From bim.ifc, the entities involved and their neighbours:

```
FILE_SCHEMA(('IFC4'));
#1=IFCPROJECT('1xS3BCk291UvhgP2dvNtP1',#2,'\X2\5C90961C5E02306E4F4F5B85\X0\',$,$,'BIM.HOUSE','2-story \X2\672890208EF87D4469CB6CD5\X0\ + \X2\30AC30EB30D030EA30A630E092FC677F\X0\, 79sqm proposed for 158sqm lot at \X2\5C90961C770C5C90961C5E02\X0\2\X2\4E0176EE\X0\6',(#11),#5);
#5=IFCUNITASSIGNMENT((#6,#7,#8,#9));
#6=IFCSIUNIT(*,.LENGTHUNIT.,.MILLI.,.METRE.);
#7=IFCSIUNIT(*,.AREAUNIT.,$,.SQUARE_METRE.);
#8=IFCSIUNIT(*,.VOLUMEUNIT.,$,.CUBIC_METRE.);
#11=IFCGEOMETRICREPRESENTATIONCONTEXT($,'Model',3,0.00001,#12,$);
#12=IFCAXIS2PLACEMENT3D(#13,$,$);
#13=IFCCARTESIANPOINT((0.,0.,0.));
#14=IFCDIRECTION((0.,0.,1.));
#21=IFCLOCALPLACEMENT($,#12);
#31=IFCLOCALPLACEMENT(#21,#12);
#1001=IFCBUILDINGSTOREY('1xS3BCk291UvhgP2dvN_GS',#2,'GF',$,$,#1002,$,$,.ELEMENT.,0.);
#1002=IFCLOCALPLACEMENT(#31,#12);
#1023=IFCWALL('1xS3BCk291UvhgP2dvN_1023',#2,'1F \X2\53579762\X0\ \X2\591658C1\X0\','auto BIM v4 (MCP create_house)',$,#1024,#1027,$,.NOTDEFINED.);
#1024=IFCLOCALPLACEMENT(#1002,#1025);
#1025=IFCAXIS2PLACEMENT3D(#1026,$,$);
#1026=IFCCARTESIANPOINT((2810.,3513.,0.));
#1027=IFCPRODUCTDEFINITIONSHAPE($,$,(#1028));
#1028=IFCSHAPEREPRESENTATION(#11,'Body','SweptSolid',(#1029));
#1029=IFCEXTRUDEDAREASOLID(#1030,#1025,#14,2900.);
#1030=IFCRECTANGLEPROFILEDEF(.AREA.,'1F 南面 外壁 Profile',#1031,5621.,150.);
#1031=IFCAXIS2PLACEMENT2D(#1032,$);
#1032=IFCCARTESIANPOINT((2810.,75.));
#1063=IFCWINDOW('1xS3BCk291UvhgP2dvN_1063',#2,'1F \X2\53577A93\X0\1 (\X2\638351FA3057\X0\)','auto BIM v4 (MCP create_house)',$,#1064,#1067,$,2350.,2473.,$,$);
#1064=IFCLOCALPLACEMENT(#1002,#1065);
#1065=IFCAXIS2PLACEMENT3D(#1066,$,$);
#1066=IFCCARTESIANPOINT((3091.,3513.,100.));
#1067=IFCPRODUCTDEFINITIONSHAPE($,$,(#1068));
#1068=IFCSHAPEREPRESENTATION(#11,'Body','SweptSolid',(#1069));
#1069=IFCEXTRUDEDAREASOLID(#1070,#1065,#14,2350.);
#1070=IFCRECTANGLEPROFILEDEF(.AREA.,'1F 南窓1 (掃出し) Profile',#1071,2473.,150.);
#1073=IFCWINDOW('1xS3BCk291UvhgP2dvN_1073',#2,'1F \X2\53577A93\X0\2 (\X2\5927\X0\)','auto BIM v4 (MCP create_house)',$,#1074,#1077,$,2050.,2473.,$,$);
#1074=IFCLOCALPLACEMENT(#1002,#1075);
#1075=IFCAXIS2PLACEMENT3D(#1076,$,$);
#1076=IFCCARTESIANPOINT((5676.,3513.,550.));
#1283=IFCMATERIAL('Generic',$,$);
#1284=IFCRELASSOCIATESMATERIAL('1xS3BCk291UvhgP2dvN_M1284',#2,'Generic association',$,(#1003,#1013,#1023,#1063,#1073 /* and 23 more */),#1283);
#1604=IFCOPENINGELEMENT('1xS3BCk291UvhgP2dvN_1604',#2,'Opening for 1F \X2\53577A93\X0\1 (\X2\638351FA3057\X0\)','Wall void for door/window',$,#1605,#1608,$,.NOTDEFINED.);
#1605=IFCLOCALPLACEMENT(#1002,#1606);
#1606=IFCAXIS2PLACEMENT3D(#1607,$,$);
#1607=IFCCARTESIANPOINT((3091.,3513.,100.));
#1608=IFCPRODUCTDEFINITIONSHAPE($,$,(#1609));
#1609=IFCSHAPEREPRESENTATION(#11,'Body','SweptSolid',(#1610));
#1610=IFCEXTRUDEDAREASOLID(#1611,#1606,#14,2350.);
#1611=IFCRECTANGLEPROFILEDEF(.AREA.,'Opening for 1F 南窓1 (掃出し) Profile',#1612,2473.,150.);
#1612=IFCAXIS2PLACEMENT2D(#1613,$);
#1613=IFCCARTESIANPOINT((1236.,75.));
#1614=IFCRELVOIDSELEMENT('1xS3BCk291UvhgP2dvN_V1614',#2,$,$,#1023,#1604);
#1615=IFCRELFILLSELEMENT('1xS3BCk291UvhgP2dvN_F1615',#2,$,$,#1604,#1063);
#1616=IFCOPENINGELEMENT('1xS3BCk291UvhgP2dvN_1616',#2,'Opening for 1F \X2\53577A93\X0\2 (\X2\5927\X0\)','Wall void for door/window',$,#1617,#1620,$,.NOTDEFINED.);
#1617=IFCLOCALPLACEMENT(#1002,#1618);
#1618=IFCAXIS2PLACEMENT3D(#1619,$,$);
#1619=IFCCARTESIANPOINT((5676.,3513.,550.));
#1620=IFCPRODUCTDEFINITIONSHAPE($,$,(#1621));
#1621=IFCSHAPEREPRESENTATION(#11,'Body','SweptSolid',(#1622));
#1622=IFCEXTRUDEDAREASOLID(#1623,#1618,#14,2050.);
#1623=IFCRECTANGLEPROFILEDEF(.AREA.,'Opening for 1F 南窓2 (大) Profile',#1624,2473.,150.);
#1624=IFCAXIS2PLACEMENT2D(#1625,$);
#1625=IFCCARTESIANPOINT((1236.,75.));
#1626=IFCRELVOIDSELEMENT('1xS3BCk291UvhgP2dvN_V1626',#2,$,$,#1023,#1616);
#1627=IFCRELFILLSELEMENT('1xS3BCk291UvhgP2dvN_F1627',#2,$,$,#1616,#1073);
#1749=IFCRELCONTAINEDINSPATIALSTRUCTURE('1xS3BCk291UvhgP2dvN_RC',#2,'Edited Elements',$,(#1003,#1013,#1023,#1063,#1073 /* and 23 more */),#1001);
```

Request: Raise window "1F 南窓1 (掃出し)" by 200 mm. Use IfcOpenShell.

```python
import numpy as np
import ifcopenshell
import ifcopenshell.api.geometry
import ifcopenshell.util.placement
import ifcopenshell.util.unit

model = ifcopenshell.open("bim.ifc")
unit_scale = ifcopenshell.util.unit.calculate_unit_scale(model)

window = model.by_guid("1xS3BCk291UvhgP2dvN_1063")
opening = window.FillsVoids[0].RelatingOpeningElement
dz = 0.2 / unit_scale

shift = np.array([0.0, 0.0, dz])
# The window is not placed relative to its opening, so move both.
for product in (opening, window):
    matrix = ifcopenshell.util.placement.get_local_placement(product.ObjectPlacement)
    matrix[:3, 3] += shift
    ifcopenshell.api.geometry.edit_object_placement(model, product=product, matrix=matrix, is_si=False)

print(f"moved by {dz * unit_scale:+.3f} m")

model.write("bim_v2.ifc")
```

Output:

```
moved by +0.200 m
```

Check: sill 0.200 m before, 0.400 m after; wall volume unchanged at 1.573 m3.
